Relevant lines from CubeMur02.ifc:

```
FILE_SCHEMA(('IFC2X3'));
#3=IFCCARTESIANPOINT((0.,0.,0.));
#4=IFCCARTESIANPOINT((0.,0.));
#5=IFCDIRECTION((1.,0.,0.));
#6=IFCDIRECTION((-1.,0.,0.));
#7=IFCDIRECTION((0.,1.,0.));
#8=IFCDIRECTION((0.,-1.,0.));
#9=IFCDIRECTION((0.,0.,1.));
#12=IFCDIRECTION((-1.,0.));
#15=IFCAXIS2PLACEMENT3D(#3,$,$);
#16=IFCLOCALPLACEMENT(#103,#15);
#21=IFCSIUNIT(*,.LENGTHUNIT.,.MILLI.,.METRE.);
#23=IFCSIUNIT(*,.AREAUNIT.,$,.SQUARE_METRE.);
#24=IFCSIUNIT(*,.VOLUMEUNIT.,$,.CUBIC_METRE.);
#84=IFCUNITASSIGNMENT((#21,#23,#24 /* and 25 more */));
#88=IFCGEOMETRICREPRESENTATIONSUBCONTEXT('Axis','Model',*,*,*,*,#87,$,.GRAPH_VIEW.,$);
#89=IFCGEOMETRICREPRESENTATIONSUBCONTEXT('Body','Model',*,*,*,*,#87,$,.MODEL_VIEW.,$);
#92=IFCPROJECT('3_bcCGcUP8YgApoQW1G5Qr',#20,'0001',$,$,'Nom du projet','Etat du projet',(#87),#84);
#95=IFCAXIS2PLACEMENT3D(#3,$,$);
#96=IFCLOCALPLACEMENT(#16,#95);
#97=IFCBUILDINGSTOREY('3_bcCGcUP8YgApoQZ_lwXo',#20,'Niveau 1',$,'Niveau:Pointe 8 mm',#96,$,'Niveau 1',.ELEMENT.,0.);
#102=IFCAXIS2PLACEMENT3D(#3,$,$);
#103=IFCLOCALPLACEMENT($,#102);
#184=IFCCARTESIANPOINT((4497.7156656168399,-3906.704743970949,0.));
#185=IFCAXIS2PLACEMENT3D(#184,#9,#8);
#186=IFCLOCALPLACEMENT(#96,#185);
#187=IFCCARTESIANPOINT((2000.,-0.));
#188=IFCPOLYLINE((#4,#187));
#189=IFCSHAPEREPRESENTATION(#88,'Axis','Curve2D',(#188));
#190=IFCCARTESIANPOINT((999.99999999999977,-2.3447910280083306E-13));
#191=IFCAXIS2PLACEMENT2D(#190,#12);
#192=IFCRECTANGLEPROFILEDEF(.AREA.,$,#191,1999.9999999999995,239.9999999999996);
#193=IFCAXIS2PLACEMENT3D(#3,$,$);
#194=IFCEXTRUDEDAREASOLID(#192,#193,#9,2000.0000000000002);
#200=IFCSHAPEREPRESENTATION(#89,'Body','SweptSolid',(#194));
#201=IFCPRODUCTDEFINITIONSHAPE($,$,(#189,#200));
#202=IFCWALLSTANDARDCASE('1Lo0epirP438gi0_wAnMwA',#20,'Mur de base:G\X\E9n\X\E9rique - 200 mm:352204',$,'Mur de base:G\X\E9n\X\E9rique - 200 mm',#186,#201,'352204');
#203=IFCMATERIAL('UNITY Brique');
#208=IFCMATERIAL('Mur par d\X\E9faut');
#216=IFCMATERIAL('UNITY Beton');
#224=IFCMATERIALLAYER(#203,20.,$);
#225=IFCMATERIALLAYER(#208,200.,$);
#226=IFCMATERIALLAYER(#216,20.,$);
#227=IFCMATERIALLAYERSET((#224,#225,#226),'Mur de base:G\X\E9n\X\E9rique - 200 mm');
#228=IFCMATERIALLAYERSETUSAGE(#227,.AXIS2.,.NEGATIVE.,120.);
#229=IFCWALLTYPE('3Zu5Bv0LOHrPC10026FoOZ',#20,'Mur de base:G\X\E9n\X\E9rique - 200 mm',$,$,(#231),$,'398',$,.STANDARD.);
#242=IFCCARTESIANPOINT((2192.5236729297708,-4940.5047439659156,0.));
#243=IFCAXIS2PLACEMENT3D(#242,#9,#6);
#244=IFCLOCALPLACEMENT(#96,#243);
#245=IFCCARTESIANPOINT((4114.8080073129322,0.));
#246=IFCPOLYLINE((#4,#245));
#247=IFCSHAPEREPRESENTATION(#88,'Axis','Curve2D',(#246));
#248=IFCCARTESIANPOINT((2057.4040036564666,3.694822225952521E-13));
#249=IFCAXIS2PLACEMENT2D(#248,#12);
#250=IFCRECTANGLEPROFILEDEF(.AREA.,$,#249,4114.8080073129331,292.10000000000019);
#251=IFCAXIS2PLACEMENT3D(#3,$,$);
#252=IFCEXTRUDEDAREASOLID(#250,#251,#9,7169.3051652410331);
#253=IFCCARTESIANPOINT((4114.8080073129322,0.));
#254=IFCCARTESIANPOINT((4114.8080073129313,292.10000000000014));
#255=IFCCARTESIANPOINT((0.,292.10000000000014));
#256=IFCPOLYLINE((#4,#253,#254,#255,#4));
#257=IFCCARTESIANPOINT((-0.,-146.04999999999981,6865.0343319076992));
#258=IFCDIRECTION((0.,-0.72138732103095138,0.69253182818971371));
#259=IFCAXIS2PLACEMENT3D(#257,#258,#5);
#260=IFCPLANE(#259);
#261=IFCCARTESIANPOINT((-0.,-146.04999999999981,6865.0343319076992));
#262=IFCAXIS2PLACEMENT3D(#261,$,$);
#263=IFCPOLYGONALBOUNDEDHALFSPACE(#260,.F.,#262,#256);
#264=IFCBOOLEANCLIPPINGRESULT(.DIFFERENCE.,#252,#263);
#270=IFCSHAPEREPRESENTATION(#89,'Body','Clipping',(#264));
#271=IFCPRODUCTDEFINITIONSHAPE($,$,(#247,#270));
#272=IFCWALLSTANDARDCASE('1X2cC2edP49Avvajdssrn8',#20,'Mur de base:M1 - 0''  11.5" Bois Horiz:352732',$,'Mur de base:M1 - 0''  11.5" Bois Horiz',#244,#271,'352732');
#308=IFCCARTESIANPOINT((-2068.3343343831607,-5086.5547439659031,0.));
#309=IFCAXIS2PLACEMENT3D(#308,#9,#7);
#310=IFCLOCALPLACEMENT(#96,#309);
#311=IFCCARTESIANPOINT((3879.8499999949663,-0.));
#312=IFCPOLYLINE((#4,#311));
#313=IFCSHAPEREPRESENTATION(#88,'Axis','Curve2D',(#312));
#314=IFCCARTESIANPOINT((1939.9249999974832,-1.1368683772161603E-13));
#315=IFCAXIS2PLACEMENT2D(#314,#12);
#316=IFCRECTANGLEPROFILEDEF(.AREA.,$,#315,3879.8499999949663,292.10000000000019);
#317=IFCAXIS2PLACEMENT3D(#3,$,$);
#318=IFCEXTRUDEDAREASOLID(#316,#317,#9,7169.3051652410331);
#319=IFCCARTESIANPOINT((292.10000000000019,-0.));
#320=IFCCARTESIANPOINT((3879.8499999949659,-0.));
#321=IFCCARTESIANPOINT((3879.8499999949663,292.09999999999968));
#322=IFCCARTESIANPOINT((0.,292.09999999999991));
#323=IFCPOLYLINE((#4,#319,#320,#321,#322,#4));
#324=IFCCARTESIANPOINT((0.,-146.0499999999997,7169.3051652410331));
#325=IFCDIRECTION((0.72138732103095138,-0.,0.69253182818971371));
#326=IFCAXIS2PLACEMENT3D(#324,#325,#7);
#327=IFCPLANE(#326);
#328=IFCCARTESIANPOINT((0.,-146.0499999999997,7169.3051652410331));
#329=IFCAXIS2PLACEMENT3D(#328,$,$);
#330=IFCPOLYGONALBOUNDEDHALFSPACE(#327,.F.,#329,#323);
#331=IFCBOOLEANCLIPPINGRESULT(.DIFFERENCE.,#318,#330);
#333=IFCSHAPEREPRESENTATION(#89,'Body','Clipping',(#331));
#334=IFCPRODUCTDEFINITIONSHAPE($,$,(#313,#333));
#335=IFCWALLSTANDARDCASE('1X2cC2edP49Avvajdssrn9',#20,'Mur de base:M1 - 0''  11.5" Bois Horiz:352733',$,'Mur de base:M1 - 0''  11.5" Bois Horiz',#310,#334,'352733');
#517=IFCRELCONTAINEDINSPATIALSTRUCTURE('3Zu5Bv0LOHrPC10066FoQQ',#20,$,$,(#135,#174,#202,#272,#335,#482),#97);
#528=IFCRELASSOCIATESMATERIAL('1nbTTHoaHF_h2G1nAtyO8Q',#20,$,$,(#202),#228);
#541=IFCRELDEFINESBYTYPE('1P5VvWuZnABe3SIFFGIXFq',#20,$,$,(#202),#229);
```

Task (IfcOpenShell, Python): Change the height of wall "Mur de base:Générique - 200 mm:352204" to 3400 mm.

```python
import ifcopenshell
import ifcopenshell.geom
import ifcopenshell.util.representation
import ifcopenshell.util.shape

model = ifcopenshell.open("CubeMur02.ifc")
settings = ifcopenshell.geom.settings()


def volume(element):
    """Net volume in cubic metres, openings subtracted."""
    shape = ifcopenshell.geom.create_shape(settings, element)
    return ifcopenshell.util.shape.get_volume(shape.geometry)


wall = model.by_guid("1Lo0epirP438gi0_wAnMwA")
before = volume(wall)

body = ifcopenshell.util.representation.get_representation(wall, "Model", "Body")
solid = body.Items[0]
old_height = solid.Depth
solid.Depth = 3400.0
after = volume(wall)

print(f"height {old_height:g} -> {solid.Depth:g}, volume {before:.3f} -> {after:.3f} m3")

model.write("CubeMur02_v2.ifc")
```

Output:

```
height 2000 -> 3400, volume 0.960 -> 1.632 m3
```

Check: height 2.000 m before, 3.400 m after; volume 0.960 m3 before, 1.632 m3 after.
